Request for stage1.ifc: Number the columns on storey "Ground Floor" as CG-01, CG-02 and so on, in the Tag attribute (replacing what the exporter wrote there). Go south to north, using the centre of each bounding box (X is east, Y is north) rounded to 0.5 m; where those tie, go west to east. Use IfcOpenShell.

First a look at what the model holds.

```python
import ifcopenshell
import ifcopenshell.util.element
import ifcopenshell.util.placement

model = ifcopenshell.open("stage1.ifc")
print(model.schema)
storey = next(s for s in model.by_type("IfcBuildingStorey") if s.Name == "Ground Floor")
columns = [e for e in ifcopenshell.util.element.get_decomposition(storey) if e.is_a("IfcColumn")]
for e in sorted(columns, key=lambda e: e.id()):
    origin = ifcopenshell.util.placement.get_local_placement(e.ObjectPlacement)[:3, 3]
    print(e.id(), e.Tag, e.Name, origin.round(2) + 0.0, sep=" | ")
```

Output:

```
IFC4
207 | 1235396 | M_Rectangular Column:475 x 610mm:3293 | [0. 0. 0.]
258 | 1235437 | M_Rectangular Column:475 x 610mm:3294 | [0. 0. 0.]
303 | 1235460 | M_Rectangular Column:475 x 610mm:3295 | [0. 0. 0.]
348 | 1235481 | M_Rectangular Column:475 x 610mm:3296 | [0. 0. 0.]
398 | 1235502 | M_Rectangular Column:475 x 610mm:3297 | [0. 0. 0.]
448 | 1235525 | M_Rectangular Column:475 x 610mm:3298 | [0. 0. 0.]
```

```python
import ifcopenshell
import ifcopenshell.geom
import ifcopenshell.util.element
import ifcopenshell.util.shape

model = ifcopenshell.open("stage1.ifc")
settings = ifcopenshell.geom.settings()
settings.set("use-world-coords", True)


def centre(element):
    shape = ifcopenshell.geom.create_shape(settings, element)
    return ifcopenshell.util.shape.get_bbox_centroid(shape.geometry)


storey = next(s for s in model.by_type("IfcBuildingStorey") if s.Name == "Ground Floor")
columns = [e for e in ifcopenshell.util.element.get_decomposition(storey) if e.is_a("IfcColumn")]

# Insertion points can sit at a corner or the storey origin, so sort by the geometry (in metres).
centres = {e: centre(e) for e in columns}
columns.sort(key=lambda e: (round(centres[e][1] / 0.5), centres[e][0]))

for i, e in enumerate(columns, start=1):
    number = f"CG-{i:02d}"
    e.Tag = number
    print(e.id(), number)

model.write("stage1_edited.ifc")
```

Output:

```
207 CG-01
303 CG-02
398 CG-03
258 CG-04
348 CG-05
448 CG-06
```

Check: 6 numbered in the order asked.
